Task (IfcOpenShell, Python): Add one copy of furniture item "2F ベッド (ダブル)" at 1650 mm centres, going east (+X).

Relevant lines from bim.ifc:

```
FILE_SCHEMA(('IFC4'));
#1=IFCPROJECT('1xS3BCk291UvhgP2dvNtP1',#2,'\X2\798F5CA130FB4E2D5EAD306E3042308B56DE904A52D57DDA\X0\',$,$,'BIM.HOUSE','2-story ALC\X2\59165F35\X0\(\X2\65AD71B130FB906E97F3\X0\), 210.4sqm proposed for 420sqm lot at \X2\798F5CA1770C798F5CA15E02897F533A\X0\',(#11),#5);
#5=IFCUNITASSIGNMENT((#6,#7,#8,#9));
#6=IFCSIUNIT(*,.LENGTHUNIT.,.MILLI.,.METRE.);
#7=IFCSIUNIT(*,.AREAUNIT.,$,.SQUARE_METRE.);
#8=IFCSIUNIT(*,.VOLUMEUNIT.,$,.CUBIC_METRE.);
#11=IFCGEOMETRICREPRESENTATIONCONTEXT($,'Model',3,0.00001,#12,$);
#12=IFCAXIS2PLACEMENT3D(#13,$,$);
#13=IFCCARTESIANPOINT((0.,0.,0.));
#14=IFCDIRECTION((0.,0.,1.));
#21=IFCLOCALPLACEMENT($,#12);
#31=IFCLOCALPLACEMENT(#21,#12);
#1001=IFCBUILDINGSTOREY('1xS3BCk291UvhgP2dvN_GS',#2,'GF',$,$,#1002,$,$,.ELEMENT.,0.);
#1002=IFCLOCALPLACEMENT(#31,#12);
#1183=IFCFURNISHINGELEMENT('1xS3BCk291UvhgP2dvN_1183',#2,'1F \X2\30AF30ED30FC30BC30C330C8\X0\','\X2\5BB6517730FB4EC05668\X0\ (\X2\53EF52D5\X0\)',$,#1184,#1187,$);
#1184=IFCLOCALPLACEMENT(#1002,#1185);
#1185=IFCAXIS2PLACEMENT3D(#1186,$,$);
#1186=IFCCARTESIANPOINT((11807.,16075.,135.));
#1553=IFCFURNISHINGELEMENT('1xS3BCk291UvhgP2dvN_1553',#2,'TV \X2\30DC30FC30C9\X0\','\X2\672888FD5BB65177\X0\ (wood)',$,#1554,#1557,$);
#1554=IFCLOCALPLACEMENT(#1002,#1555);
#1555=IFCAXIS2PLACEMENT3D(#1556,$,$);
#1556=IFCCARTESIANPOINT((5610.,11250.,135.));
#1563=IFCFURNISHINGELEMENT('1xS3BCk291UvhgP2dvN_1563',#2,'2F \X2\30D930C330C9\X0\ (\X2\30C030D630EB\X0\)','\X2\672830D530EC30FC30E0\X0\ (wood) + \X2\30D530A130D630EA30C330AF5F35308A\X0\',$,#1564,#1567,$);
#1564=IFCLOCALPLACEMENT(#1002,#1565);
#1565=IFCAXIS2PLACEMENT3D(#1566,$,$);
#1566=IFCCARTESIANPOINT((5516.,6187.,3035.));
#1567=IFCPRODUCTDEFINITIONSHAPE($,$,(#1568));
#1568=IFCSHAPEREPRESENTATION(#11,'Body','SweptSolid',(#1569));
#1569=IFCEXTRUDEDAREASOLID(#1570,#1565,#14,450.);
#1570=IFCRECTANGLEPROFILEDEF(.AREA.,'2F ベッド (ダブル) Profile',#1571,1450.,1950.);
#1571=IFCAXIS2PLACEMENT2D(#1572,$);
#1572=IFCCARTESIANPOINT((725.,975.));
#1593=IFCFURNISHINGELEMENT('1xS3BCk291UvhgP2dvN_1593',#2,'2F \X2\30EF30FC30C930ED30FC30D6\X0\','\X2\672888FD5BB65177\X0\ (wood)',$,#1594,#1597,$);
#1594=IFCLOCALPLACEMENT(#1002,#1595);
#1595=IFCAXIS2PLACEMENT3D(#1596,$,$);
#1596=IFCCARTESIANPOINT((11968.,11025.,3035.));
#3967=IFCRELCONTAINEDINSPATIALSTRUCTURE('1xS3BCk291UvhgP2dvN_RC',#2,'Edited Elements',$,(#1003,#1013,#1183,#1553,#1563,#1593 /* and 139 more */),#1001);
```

```python
import numpy as np
import ifcopenshell
import ifcopenshell.api.geometry
import ifcopenshell.api.root
import ifcopenshell.util.element
import ifcopenshell.util.placement
import ifcopenshell.util.unit

model = ifcopenshell.open("bim.ifc")
unit_scale = ifcopenshell.util.unit.calculate_unit_scale(model)


def reuse_history(source, copy):
    """copy_class also copies each property set's owner history, people and application; keep the originals."""
    for rel in copy.IsDefinedBy:
        if rel.is_a("IfcRelDefinesByProperties") and (history := rel.RelatingPropertyDefinition.OwnerHistory):
            rel.RelatingPropertyDefinition.OwnerHistory = source.OwnerHistory
            ifcopenshell.util.element.remove_deep2(model, history)


source = model.by_id(1563)
base = ifcopenshell.util.placement.get_local_placement(source.ObjectPlacement)
step = np.array([1.0, 0.0, 0.0]) * 1.65 / unit_scale

for i in range(1, 2):
    copy = ifcopenshell.api.root.copy_class(model, product=source)
    copy.Representation = ifcopenshell.util.element.copy_deep(
        model, source.Representation, exclude=["IfcGeometricRepresentationContext", "IfcRepresentationMap"]
    )
    reuse_history(source, copy)
    matrix = base.copy()
    matrix[:3, 3] += i * step
    print("added at", matrix[:3, 3].round(3) + 0.0)
    ifcopenshell.api.geometry.edit_object_placement(model, product=copy, matrix=matrix, is_si=False)

model.write("bim-out.ifc")
```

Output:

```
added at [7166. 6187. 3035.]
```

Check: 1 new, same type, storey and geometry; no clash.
